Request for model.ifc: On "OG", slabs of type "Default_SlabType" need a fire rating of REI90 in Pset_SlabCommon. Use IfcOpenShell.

First a look at what the model holds.

```python
import ifcopenshell
import ifcopenshell.util.element

model = ifcopenshell.open("model.ifc")
print(model.schema)
storey = next(s for s in model.by_type("IfcBuildingStorey") if s.Name == "OG")
slabs = [e for e in ifcopenshell.util.element.get_decomposition(storey) if e.is_a("IfcSlab")]
seen = {}
for e in slabs:
    element_type = ifcopenshell.util.element.get_type(e)
    key = (element_type.Name if element_type != e and element_type else None, ifcopenshell.util.element.get_pset(e, "Pset_SlabCommon", "FireRating"))
    seen[key] = seen.get(key, 0) + 1
for (name, value), count in sorted(seen.items(), key=str):
    print(count, "x", name, "|", value)
```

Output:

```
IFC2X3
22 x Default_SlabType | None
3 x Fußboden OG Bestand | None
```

```python
import ifcopenshell
import ifcopenshell.api.pset
import ifcopenshell.util.element

model = ifcopenshell.open("model.ifc")

storey = next(s for s in model.by_type("IfcBuildingStorey") if s.Name == "OG")
slabs = [e for e in ifcopenshell.util.element.get_decomposition(storey) if e.is_a("IfcSlab")]

count = 0
for e in slabs:
    element_type = ifcopenshell.util.element.get_type(e)
    if element_type in (None, e) or element_type.Name != "Default_SlabType":
        continue
    # add_pset returns the element's existing set when there is one.
    pset = ifcopenshell.api.pset.add_pset(model, product=e, name="Pset_SlabCommon")
    ifcopenshell.api.pset.edit_pset(model, pset=pset, properties={"FireRating": "REI90"})
    count += 1

print(count, "slabs updated")

model.write("model_updated.ifc")
```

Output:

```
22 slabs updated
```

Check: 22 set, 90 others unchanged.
